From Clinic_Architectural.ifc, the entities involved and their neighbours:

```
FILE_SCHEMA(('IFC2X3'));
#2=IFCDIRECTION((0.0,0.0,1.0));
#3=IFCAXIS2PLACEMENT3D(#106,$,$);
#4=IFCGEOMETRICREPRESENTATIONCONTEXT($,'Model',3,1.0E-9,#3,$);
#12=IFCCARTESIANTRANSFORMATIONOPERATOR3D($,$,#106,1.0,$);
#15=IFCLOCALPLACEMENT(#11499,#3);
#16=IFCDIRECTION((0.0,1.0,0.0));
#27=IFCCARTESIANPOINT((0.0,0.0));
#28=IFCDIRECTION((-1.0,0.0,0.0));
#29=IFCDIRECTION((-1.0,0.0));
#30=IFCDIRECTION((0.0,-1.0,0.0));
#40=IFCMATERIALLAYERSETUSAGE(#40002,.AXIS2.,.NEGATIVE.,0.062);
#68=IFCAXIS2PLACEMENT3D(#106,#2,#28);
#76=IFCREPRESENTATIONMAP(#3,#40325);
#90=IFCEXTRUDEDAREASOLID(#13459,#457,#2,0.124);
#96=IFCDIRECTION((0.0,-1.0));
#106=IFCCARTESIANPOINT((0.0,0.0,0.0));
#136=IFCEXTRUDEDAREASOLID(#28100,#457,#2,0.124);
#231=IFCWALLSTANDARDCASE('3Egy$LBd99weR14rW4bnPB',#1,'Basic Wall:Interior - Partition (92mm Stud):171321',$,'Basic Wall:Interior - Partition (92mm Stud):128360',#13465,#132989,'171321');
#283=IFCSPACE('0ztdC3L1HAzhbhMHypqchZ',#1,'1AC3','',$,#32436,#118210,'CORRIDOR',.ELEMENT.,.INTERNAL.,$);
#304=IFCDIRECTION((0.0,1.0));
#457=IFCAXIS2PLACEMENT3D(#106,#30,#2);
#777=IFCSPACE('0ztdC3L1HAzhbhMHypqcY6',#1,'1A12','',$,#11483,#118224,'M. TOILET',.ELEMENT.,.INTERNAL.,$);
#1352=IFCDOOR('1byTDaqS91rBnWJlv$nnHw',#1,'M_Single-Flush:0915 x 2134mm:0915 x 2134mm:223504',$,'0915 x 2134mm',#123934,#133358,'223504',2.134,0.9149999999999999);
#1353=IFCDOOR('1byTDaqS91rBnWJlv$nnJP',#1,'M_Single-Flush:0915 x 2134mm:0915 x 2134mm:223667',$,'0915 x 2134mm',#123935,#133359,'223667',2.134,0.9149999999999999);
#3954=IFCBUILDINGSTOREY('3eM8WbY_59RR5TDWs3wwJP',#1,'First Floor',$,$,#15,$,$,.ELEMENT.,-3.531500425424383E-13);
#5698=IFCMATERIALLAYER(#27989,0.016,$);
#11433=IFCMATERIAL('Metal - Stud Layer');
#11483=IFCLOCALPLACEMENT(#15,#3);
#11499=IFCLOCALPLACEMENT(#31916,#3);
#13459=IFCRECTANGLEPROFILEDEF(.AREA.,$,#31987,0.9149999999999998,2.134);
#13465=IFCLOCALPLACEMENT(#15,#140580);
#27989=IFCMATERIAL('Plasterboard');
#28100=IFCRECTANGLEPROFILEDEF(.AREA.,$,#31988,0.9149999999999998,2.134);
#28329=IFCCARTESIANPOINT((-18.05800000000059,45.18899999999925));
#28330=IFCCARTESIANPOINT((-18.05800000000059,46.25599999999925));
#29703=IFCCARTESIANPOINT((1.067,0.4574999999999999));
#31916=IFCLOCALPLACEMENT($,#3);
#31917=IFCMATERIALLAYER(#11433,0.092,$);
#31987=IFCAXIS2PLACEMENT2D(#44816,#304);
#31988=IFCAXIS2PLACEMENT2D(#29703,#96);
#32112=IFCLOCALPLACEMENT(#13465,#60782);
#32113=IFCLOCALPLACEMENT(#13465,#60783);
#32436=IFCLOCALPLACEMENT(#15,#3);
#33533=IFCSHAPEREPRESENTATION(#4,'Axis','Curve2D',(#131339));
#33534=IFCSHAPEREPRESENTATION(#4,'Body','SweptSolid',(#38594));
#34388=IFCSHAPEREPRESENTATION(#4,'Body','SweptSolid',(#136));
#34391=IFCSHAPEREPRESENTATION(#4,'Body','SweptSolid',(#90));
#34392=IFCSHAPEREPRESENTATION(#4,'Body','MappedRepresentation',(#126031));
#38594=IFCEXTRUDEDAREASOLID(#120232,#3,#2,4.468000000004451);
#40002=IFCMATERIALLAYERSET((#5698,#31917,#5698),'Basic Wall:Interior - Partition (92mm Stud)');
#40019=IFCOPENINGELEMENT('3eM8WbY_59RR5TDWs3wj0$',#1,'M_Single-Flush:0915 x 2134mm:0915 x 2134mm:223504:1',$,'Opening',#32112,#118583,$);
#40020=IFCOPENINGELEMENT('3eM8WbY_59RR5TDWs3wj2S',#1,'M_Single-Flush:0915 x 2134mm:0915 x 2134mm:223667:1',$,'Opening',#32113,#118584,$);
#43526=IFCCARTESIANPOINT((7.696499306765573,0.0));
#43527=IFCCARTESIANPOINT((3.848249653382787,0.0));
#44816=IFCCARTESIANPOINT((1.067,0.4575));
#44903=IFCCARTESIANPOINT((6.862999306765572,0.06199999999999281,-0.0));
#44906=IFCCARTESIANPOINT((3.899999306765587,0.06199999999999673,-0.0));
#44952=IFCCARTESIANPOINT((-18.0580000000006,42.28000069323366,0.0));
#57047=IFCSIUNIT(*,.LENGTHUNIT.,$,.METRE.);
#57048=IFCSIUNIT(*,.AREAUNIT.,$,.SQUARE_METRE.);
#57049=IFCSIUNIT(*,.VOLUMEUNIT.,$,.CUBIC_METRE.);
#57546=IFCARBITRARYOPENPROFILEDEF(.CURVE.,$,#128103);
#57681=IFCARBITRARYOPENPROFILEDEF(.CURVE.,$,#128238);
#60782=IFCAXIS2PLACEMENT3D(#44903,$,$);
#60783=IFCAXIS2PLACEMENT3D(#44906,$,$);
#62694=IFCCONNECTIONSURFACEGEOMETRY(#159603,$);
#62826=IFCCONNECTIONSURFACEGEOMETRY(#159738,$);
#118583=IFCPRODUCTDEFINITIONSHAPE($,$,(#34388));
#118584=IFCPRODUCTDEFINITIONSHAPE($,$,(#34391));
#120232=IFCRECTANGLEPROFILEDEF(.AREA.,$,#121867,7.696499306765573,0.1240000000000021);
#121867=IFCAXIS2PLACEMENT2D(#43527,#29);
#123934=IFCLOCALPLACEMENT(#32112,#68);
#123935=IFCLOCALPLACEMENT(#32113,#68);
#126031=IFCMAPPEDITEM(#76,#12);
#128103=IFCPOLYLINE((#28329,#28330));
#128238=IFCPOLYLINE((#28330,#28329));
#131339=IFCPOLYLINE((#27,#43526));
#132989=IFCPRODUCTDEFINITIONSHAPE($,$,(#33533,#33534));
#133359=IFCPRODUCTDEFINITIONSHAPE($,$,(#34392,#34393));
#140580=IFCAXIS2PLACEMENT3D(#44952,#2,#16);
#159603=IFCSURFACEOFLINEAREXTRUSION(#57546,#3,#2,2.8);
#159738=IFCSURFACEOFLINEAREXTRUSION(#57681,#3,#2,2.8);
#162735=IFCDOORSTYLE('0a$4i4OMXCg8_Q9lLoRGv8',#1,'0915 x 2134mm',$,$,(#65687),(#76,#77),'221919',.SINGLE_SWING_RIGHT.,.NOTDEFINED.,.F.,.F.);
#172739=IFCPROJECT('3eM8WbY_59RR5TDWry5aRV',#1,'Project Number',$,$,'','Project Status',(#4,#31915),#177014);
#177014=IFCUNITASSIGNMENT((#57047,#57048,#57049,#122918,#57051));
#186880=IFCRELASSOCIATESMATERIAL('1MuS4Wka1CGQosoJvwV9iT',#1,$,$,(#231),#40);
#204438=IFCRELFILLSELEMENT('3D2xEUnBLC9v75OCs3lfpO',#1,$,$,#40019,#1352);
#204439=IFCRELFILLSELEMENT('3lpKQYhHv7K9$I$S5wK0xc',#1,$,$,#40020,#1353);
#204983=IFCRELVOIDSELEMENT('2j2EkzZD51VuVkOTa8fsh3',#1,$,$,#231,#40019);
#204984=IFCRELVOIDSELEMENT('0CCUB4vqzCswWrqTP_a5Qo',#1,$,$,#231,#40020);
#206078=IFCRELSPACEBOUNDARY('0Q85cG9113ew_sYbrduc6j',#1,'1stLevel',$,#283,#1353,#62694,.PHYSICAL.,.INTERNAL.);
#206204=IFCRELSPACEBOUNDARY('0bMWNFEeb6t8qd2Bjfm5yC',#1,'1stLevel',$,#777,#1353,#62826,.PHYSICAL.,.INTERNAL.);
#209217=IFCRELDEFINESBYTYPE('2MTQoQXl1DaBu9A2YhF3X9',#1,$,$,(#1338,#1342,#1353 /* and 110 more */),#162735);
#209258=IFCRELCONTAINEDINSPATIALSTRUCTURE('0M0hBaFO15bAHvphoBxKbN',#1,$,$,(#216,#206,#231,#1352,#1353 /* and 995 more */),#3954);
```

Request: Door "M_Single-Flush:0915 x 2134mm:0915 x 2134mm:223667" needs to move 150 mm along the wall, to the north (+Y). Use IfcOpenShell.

```python
import numpy as np
import ifcopenshell
import ifcopenshell.api.geometry
import ifcopenshell.util.placement
import ifcopenshell.util.unit

model = ifcopenshell.open("Clinic_Architectural.ifc")
unit_scale = ifcopenshell.util.unit.calculate_unit_scale(model)

door = model.by_guid("1byTDaqS91rBnWJlv$nnJP")
opening = door.FillsVoids[0].RelatingOpeningElement
wall = opening.VoidsElements[0].RelatingBuildingElement

wall_matrix = ifcopenshell.util.placement.get_local_placement(wall.ObjectPlacement)
shift = wall_matrix[:3, 0] * 0.15 / unit_scale
before = ifcopenshell.util.placement.get_local_placement(door.ObjectPlacement)[:3, 3].copy()

# The door is placed relative to its opening, so it follows when the opening moves.
matrix = ifcopenshell.util.placement.get_local_placement(opening.ObjectPlacement)
matrix[:3, 3] += shift
ifcopenshell.api.geometry.edit_object_placement(
    model, product=opening, matrix=matrix, is_si=False, should_transform_children=True
)

# Space boundary surfaces are stored in each space's coordinates; move them too.
for rel in door.ProvidesBoundaries:
    if not rel.ConnectionGeometry:
        continue
    surface = rel.ConnectionGeometry.SurfaceOnRelatingElement
    space_matrix = ifcopenshell.util.placement.get_local_placement(rel.RelatingSpace.ObjectPlacement)
    point = np.array(surface.Position.Location.Coordinates) + space_matrix[:3, :3].T @ shift
    surface.Position = model.createIfcAxis2Placement3D(
        model.createIfcCartesianPoint(point.tolist()), surface.Position.Axis, surface.Position.RefDirection
    )

after = ifcopenshell.util.placement.get_local_placement(door.ObjectPlacement)[:3, 3]
print("door moved by", (after - before).round(3) + 0.0)

model.write("Clinic_Architectural_rev.ifc")
```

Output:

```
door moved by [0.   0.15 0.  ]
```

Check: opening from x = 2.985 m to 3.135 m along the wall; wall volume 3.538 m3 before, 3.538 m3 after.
